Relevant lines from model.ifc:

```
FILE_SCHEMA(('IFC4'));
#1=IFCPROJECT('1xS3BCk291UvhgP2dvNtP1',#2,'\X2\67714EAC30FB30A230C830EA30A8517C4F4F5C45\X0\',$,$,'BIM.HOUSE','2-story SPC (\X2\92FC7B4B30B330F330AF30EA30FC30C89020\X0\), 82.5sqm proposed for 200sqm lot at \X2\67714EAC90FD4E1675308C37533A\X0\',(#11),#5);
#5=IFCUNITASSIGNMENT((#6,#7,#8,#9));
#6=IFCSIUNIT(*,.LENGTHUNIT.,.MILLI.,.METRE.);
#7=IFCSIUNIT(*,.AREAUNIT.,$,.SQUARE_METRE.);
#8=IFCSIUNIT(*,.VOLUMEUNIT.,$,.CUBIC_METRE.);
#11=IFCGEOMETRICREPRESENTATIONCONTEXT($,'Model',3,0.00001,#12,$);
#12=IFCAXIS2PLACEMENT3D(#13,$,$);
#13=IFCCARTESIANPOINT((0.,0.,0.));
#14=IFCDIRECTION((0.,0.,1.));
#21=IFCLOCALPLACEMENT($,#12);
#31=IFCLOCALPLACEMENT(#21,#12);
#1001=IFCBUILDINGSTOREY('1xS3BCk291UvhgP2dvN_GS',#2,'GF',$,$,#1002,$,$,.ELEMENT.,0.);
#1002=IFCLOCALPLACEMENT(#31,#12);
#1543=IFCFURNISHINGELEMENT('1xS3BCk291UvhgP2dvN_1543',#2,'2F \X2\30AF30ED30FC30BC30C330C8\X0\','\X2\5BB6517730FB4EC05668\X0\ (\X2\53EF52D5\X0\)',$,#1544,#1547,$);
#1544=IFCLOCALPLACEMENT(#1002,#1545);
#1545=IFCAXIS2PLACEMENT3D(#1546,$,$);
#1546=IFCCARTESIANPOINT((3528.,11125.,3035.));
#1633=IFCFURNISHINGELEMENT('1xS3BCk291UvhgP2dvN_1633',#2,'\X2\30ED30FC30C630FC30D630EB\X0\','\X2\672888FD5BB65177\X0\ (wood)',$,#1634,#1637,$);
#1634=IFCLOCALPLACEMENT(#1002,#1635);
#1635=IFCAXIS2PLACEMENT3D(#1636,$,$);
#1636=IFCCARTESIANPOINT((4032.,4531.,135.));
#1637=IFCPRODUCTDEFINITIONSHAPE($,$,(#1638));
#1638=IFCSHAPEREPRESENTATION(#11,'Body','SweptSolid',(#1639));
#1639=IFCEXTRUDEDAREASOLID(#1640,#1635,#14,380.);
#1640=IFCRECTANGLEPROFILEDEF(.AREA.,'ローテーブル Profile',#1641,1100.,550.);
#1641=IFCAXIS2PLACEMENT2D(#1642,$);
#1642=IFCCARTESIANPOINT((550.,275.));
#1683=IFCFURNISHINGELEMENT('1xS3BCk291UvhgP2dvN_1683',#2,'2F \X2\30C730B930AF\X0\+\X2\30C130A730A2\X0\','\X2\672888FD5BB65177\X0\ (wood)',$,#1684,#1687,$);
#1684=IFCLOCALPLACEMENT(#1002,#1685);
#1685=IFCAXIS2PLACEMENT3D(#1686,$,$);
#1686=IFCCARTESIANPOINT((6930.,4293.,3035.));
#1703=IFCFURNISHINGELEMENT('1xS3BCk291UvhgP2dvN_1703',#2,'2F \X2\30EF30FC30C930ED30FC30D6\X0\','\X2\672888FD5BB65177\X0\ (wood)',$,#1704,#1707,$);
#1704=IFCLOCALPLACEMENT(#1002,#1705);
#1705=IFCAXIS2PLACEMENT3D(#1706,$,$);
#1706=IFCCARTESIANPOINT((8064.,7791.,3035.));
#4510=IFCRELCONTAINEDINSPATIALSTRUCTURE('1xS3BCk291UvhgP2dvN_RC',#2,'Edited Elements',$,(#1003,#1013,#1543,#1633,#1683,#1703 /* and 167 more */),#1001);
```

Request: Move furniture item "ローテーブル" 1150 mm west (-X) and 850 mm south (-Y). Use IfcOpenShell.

```python
import ifcopenshell
import ifcopenshell.api.geometry
import ifcopenshell.util.placement
import ifcopenshell.util.unit

model = ifcopenshell.open("model.ifc")
unit_scale = ifcopenshell.util.unit.calculate_unit_scale(model)

item = model.by_guid("1xS3BCk291UvhgP2dvN_1633")
matrix = ifcopenshell.util.placement.get_local_placement(item.ObjectPlacement)
matrix[0, 3] -= 1.15 / unit_scale
matrix[1, 3] -= 0.85 / unit_scale
ifcopenshell.api.geometry.edit_object_placement(model, product=item, matrix=matrix, is_si=False)

print(ifcopenshell.util.placement.get_local_placement(item.ObjectPlacement).round(3) + 0.0)

model.write("model_rev.ifc")
```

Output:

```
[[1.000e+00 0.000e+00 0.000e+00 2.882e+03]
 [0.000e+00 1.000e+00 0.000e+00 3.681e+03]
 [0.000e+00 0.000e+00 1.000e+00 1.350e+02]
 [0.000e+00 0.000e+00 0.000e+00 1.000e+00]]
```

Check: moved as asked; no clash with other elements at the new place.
